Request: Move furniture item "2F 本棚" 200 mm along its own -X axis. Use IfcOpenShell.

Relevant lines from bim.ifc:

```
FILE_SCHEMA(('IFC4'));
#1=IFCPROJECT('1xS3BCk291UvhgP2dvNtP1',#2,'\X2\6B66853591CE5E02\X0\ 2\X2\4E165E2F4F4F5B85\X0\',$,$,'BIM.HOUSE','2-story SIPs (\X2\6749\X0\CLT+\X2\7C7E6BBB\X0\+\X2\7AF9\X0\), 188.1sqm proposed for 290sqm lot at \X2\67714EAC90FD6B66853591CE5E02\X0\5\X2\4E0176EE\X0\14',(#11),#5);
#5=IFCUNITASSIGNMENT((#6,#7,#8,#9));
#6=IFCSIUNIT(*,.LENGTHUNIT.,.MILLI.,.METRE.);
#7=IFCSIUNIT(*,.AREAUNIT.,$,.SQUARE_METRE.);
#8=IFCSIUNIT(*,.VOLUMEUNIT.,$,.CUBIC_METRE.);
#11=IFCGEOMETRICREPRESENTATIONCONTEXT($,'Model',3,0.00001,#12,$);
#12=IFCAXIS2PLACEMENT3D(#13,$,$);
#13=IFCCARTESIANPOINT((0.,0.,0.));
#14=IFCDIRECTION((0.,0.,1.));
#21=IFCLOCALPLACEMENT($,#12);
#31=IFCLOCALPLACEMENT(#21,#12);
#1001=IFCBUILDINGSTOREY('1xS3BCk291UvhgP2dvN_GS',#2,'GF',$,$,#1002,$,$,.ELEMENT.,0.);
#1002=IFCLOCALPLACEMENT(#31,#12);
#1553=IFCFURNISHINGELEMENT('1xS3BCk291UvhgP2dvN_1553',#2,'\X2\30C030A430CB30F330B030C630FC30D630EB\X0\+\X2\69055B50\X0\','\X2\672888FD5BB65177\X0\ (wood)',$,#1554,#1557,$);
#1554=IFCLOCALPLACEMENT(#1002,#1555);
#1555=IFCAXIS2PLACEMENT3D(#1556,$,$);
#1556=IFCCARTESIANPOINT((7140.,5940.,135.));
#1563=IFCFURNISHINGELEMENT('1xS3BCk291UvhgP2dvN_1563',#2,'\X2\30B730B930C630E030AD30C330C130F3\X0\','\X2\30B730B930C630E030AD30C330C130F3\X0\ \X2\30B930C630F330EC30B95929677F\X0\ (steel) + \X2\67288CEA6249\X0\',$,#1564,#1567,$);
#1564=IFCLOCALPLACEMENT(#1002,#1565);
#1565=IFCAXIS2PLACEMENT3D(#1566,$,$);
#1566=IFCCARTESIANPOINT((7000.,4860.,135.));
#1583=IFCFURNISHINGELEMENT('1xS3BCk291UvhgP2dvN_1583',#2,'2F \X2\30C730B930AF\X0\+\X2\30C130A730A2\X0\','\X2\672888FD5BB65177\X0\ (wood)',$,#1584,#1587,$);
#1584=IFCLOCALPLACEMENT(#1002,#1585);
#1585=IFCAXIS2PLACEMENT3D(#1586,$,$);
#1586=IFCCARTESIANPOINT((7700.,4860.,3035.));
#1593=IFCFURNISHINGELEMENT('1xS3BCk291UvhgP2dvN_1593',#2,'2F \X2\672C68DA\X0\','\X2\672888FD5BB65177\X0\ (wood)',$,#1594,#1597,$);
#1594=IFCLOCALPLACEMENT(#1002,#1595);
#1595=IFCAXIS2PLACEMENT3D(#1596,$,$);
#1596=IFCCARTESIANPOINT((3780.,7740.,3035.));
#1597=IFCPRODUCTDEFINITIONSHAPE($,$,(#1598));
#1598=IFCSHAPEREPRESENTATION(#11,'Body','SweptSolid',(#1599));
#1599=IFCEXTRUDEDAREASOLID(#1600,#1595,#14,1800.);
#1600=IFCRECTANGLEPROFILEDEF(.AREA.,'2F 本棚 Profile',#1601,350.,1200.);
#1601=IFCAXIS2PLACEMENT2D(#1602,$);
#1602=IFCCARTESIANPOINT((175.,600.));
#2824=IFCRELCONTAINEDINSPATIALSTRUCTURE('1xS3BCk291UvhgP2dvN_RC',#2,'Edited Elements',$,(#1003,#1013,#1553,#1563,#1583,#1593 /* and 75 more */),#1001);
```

```python
import ifcopenshell
import ifcopenshell.api.geometry
import ifcopenshell.util.placement
import ifcopenshell.util.unit

model = ifcopenshell.open("bim.ifc")
unit_scale = ifcopenshell.util.unit.calculate_unit_scale(model)

item = model.by_id(1593)
matrix = ifcopenshell.util.placement.get_local_placement(item.ObjectPlacement)
matrix[:3, 3] -= matrix[:3, 0] * 0.2 / unit_scale
ifcopenshell.api.geometry.edit_object_placement(model, product=item, matrix=matrix, is_si=False)

print(ifcopenshell.util.placement.get_local_placement(item.ObjectPlacement).round(3) + 0.0)

model.write("bim_rev.ifc")
```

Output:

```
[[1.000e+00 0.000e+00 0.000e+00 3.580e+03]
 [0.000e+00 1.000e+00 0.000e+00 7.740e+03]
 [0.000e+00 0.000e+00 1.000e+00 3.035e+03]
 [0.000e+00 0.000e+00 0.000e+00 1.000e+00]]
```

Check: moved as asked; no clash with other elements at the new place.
